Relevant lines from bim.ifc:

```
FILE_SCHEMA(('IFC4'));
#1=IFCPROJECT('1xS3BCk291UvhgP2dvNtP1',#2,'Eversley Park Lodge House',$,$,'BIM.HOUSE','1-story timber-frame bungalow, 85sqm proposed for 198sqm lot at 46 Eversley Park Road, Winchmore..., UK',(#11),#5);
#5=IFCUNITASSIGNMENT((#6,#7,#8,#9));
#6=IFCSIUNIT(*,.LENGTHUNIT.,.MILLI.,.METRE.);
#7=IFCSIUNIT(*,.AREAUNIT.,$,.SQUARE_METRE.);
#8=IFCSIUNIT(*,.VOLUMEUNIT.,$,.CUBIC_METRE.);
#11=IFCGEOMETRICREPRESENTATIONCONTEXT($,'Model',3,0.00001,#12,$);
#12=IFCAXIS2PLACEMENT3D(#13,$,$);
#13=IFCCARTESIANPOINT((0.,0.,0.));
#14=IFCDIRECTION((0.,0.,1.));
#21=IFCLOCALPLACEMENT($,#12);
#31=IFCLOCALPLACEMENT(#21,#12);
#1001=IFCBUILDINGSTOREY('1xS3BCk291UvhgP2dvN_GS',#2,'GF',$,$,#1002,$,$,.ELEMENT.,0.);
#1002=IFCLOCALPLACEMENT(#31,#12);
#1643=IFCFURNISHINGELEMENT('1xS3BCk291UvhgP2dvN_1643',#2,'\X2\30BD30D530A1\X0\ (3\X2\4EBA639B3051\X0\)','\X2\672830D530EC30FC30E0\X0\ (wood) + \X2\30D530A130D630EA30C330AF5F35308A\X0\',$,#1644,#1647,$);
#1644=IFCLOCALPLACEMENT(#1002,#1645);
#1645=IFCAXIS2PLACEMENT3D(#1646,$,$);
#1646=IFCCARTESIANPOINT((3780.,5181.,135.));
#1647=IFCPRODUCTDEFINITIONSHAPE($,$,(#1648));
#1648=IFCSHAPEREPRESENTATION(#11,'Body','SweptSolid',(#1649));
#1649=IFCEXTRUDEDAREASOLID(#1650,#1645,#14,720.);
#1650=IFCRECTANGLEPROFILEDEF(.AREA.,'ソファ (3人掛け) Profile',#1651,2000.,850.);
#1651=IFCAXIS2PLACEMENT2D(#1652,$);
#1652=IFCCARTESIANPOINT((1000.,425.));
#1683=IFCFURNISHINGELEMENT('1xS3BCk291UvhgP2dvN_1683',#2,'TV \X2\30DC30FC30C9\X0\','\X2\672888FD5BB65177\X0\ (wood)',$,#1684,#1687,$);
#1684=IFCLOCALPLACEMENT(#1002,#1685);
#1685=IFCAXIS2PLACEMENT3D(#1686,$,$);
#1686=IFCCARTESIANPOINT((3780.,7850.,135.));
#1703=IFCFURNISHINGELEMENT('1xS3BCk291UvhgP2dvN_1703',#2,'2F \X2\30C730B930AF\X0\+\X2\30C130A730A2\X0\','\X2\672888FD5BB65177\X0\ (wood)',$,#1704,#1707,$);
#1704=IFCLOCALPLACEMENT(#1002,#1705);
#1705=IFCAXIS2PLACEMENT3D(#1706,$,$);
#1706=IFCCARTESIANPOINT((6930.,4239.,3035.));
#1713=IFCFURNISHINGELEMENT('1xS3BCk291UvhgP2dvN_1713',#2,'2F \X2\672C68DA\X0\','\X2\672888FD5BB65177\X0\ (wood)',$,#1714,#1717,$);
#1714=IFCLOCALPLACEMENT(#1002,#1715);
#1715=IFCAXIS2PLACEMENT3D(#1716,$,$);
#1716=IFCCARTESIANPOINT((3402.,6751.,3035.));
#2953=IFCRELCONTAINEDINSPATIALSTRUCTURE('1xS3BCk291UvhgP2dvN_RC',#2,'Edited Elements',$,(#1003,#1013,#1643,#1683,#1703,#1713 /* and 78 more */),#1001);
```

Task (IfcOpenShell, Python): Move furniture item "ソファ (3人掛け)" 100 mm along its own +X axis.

```python
import ifcopenshell
import ifcopenshell.api.geometry
import ifcopenshell.util.placement

model = ifcopenshell.open("bim.ifc")

item = model.by_guid("1xS3BCk291UvhgP2dvN_1643")
matrix = ifcopenshell.util.placement.get_local_placement(item.ObjectPlacement)
matrix[:3, 3] += matrix[:3, 0] * 100.0
ifcopenshell.api.geometry.edit_object_placement(model, product=item, matrix=matrix, is_si=False)

print(ifcopenshell.util.placement.get_local_placement(item.ObjectPlacement).round(3) + 0.0)

model.write("bim-out.ifc")
```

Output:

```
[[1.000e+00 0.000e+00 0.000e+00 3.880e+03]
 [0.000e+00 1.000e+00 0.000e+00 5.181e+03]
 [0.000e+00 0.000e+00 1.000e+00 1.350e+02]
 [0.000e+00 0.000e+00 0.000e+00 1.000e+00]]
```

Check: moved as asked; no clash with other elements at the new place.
